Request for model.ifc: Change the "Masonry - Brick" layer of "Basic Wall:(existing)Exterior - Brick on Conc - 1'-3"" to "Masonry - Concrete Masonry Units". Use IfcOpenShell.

First a look at what the model holds.

```python
import ifcopenshell
import ifcopenshell.util.element

model = ifcopenshell.open("model.ifc")
print(model.schema)
for layer_set in model.by_type("IfcMaterialLayerSet"):
    if layer_set.LayerSetName == 'Basic Wall:(existing)Exterior - Brick on Conc - 1\'-3"':
        for layer in layer_set.MaterialLayers:
            print(layer.id(), layer.Material and layer.Material.Name, layer.LayerThickness, sep=" | ")
        print(len(ifcopenshell.util.element.get_elements_by_material(model, layer_set)), "elements and types use it")
print(sorted(m.Name for m in model.by_type("IfcMaterial") if m.Name)[:60])
```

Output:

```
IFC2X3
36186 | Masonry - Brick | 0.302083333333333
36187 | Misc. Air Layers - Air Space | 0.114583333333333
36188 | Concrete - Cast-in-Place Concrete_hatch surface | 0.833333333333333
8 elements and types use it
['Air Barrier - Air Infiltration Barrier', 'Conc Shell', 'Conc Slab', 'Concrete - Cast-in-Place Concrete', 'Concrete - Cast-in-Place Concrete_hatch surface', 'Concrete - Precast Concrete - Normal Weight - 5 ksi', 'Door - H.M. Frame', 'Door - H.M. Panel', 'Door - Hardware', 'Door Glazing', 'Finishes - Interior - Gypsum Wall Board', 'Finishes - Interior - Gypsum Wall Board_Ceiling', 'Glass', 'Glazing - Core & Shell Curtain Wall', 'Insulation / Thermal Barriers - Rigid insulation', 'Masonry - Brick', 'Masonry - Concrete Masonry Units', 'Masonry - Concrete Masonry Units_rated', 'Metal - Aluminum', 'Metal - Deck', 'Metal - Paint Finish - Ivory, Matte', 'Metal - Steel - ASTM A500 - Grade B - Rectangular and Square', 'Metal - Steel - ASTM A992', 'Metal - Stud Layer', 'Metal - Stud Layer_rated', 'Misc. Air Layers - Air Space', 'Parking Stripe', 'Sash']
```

```python
import ifcopenshell
import ifcopenshell.api.material

model = ifcopenshell.open("model.ifc")

layer_set = next(s for s in model.by_type("IfcMaterialLayerSet") if s.LayerSetName == 'Basic Wall:(existing)Exterior - Brick on Conc - 1\'-3"')
layer = next(l for l in layer_set.MaterialLayers if l.Material and l.Material.Name == "Masonry - Brick")
material = next(m for m in model.by_type("IfcMaterial") if m.Name == "Masonry - Concrete Masonry Units")

# Point this one layer at the other material; renaming the old one would change it everywhere.
ifcopenshell.api.material.edit_layer(model, layer=layer, attributes={}, material=material)

print([l.Material.Name if l.Material else None for l in layer_set.MaterialLayers])

model.write("model_updated.ifc")
```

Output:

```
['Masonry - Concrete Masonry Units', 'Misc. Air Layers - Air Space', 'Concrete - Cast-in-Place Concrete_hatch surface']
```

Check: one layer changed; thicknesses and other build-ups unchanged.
